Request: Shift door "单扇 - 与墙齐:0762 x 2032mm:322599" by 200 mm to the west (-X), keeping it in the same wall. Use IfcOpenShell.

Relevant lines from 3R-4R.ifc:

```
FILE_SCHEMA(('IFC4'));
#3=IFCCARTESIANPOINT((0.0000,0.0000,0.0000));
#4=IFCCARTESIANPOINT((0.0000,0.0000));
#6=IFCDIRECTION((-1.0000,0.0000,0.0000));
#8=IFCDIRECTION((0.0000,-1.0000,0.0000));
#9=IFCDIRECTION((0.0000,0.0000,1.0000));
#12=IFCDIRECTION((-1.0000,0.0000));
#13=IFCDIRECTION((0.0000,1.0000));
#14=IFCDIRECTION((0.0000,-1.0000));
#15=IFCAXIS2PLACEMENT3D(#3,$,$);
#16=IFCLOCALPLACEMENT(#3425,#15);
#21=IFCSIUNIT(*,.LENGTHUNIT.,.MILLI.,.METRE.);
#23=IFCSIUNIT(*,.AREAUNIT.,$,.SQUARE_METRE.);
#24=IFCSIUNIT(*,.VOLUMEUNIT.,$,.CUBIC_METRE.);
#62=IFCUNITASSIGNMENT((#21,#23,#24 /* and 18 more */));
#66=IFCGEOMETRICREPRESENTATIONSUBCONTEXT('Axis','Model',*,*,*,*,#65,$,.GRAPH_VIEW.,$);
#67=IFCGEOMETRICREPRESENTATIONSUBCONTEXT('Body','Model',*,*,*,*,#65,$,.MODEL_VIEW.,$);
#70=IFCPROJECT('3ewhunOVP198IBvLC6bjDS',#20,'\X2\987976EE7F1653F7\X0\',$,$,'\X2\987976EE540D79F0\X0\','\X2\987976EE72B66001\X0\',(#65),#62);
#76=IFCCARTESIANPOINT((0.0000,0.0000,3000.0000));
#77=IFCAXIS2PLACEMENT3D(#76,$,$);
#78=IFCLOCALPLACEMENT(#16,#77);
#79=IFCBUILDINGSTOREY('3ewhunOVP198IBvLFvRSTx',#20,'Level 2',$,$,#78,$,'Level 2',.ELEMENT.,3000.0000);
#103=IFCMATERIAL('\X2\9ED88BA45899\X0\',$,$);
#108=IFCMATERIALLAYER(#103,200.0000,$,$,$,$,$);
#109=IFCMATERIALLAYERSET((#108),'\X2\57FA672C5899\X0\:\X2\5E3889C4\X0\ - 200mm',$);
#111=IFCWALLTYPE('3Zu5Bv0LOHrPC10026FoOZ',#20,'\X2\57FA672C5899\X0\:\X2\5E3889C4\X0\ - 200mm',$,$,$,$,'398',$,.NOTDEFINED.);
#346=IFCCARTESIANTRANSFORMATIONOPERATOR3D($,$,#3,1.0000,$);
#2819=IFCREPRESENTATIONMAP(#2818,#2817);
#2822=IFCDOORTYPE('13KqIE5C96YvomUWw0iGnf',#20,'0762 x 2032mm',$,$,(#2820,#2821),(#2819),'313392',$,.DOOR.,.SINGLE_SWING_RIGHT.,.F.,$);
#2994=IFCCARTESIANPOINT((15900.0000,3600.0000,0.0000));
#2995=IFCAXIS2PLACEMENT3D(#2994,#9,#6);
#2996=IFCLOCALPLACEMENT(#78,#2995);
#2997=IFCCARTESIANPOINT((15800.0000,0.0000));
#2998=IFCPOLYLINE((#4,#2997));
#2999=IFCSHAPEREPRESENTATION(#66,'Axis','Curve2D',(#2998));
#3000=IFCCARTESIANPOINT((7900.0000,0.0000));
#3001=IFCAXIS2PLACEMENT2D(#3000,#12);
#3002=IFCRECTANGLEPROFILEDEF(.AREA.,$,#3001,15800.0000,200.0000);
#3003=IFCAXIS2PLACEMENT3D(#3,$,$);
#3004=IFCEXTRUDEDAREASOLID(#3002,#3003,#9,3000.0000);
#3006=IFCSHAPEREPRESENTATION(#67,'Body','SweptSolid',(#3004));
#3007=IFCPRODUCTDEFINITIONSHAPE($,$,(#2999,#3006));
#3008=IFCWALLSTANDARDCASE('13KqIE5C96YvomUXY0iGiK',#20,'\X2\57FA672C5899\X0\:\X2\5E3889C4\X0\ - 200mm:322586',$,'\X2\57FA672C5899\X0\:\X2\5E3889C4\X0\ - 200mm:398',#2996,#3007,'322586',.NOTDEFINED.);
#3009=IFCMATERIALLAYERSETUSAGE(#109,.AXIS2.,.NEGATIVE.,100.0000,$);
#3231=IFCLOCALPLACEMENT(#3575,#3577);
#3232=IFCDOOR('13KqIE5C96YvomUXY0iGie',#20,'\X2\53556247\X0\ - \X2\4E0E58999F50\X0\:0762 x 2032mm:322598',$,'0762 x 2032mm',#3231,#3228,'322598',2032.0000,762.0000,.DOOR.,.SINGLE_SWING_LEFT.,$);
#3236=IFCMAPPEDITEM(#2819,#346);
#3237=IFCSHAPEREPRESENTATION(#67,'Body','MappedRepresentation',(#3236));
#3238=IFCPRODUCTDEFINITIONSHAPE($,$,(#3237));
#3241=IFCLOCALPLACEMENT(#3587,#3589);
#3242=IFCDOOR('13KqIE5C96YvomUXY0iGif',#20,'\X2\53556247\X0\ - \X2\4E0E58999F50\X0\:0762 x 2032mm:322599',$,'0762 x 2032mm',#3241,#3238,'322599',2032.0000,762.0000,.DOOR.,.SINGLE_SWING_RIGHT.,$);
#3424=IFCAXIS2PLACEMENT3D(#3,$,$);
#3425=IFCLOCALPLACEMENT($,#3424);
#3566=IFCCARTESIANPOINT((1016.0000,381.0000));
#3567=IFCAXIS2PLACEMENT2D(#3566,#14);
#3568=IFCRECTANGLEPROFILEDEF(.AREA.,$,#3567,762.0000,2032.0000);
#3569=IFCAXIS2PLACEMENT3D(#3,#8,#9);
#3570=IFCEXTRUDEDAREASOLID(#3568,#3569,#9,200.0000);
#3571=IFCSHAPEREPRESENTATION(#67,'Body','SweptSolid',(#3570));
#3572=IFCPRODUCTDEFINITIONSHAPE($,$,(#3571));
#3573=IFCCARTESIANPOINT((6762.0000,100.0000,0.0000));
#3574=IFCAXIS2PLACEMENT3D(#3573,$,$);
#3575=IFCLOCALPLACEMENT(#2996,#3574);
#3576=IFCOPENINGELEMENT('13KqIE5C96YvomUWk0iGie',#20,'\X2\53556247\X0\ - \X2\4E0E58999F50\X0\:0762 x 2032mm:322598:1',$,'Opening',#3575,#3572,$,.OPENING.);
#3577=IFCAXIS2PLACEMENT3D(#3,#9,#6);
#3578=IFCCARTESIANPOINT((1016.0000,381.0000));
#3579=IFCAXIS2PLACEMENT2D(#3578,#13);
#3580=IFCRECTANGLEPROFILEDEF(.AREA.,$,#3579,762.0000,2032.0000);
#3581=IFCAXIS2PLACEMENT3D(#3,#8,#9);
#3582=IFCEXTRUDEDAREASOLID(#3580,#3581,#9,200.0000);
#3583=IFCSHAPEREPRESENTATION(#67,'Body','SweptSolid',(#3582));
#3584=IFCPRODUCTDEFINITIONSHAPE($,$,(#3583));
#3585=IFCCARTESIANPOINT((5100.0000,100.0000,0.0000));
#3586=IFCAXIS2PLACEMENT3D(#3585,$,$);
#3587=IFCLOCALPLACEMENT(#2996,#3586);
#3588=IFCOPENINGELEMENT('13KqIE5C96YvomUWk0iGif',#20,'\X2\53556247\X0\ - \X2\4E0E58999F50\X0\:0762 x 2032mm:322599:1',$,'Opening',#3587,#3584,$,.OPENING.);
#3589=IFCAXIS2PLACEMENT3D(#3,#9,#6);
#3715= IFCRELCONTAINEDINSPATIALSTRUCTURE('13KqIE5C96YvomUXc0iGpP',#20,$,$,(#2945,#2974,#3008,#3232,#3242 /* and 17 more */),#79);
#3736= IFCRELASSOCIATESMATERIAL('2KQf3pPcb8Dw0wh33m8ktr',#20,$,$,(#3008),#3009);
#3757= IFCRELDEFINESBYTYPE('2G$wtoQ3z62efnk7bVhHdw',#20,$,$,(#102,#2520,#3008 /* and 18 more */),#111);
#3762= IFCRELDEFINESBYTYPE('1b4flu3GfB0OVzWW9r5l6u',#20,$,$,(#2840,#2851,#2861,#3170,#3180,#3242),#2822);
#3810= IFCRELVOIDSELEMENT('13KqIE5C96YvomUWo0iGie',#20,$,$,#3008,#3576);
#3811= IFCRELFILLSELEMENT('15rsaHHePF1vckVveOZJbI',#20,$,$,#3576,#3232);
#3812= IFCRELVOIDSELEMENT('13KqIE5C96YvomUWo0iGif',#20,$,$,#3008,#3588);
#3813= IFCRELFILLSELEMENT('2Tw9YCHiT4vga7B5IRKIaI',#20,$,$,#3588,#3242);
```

```python
import ifcopenshell
import ifcopenshell.api.geometry
import ifcopenshell.util.placement

model = ifcopenshell.open("3R-4R.ifc")

door = model.by_id(3242)
opening = door.FillsVoids[0].RelatingOpeningElement
wall = opening.VoidsElements[0].RelatingBuildingElement

wall_matrix = ifcopenshell.util.placement.get_local_placement(wall.ObjectPlacement)
shift = wall_matrix[:3, 0] * 200.0
before = ifcopenshell.util.placement.get_local_placement(door.ObjectPlacement)[:3, 3].copy()

# The door is placed relative to its opening, so it follows when the opening moves.
matrix = ifcopenshell.util.placement.get_local_placement(opening.ObjectPlacement)
matrix[:3, 3] += shift
ifcopenshell.api.geometry.edit_object_placement(
    model, product=opening, matrix=matrix, is_si=False, should_transform_children=True
)

after = ifcopenshell.util.placement.get_local_placement(door.ObjectPlacement)[:3, 3]
print("door moved by", (after - before).round(3) + 0.0)

model.write("3R-4R_v2.ifc")
```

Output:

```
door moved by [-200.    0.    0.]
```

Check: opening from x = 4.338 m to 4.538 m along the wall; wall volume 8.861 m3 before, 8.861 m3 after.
